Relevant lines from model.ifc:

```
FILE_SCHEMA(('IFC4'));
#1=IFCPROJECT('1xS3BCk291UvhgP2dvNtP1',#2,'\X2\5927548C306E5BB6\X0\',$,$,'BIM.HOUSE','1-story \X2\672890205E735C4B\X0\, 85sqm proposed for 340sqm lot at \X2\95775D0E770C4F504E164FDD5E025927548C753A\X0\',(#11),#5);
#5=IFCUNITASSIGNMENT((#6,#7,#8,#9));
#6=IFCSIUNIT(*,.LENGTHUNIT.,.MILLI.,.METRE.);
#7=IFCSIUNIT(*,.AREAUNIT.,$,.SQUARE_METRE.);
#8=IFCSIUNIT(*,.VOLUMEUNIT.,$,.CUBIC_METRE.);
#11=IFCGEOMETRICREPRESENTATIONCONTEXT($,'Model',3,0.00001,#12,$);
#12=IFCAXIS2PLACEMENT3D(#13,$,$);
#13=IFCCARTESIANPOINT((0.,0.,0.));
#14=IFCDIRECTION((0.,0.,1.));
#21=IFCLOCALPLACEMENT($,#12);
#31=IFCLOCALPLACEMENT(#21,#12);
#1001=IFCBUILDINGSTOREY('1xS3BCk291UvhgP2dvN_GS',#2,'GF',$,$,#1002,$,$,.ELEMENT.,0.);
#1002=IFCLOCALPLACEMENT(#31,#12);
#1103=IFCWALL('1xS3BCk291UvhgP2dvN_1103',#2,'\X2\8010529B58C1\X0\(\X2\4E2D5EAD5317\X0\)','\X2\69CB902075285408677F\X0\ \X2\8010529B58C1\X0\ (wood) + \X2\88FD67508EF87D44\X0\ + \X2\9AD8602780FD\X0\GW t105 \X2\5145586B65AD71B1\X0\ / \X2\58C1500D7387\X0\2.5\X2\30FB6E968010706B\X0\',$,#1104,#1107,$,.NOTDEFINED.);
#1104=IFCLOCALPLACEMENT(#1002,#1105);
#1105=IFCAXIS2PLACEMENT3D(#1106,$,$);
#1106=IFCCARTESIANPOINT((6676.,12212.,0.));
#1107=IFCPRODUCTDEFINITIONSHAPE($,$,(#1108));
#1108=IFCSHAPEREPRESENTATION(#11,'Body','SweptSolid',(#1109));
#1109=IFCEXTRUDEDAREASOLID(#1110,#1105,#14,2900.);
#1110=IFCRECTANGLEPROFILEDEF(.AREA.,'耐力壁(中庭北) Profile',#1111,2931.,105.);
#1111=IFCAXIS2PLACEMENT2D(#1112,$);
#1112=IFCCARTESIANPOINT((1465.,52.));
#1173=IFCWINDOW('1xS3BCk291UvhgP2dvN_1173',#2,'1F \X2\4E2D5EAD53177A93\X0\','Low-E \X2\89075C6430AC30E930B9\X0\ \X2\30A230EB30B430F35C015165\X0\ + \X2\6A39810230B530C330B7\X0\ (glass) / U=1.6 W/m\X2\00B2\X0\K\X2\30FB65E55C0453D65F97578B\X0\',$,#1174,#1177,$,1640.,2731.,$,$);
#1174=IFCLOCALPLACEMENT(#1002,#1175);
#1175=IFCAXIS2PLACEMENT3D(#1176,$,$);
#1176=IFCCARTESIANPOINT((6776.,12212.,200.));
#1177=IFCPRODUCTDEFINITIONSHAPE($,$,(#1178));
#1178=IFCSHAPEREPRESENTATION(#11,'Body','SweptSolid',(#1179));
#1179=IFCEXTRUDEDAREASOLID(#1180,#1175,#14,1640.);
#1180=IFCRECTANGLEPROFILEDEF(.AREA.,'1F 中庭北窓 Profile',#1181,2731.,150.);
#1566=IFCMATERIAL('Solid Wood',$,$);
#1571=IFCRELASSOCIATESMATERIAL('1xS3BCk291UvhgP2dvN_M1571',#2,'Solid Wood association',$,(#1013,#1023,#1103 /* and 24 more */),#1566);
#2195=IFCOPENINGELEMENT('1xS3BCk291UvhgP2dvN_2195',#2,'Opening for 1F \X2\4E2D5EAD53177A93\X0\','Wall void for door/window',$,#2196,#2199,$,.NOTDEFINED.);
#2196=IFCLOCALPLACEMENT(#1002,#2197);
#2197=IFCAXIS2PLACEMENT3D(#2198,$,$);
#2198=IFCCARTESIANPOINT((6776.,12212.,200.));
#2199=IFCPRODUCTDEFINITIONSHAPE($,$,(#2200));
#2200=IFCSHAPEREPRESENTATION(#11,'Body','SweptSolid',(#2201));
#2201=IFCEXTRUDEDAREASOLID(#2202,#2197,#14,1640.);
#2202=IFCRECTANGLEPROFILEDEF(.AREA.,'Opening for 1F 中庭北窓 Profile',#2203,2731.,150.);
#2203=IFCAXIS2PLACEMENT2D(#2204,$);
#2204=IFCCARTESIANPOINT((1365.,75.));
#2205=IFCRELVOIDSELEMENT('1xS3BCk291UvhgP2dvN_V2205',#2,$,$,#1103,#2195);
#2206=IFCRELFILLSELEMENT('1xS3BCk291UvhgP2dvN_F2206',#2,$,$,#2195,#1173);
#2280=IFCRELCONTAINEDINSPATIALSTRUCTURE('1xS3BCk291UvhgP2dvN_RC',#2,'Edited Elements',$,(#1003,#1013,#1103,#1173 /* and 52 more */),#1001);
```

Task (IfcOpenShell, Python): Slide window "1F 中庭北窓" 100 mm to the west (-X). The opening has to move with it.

```python
import ifcopenshell
import ifcopenshell.api.geometry
import ifcopenshell.util.placement
import ifcopenshell.util.unit

model = ifcopenshell.open("model.ifc")
unit_scale = ifcopenshell.util.unit.calculate_unit_scale(model)

window = model.by_guid("1xS3BCk291UvhgP2dvN_1173")
opening = window.FillsVoids[0].RelatingOpeningElement
wall = opening.VoidsElements[0].RelatingBuildingElement

wall_matrix = ifcopenshell.util.placement.get_local_placement(wall.ObjectPlacement)
shift = wall_matrix[:3, 0] * -0.1 / unit_scale
before = ifcopenshell.util.placement.get_local_placement(window.ObjectPlacement)[:3, 3].copy()

# The window is not placed relative to its opening, so move both.
for product in (opening, window):
    matrix = ifcopenshell.util.placement.get_local_placement(product.ObjectPlacement)
    matrix[:3, 3] += shift
    ifcopenshell.api.geometry.edit_object_placement(model, product=product, matrix=matrix, is_si=False)

after = ifcopenshell.util.placement.get_local_placement(window.ObjectPlacement)[:3, 3]
print("window moved by", (after - before).round(3) + 0.0)

model.write("model_v2.ifc")
```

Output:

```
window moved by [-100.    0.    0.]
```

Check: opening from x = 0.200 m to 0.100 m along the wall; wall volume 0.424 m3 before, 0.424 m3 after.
